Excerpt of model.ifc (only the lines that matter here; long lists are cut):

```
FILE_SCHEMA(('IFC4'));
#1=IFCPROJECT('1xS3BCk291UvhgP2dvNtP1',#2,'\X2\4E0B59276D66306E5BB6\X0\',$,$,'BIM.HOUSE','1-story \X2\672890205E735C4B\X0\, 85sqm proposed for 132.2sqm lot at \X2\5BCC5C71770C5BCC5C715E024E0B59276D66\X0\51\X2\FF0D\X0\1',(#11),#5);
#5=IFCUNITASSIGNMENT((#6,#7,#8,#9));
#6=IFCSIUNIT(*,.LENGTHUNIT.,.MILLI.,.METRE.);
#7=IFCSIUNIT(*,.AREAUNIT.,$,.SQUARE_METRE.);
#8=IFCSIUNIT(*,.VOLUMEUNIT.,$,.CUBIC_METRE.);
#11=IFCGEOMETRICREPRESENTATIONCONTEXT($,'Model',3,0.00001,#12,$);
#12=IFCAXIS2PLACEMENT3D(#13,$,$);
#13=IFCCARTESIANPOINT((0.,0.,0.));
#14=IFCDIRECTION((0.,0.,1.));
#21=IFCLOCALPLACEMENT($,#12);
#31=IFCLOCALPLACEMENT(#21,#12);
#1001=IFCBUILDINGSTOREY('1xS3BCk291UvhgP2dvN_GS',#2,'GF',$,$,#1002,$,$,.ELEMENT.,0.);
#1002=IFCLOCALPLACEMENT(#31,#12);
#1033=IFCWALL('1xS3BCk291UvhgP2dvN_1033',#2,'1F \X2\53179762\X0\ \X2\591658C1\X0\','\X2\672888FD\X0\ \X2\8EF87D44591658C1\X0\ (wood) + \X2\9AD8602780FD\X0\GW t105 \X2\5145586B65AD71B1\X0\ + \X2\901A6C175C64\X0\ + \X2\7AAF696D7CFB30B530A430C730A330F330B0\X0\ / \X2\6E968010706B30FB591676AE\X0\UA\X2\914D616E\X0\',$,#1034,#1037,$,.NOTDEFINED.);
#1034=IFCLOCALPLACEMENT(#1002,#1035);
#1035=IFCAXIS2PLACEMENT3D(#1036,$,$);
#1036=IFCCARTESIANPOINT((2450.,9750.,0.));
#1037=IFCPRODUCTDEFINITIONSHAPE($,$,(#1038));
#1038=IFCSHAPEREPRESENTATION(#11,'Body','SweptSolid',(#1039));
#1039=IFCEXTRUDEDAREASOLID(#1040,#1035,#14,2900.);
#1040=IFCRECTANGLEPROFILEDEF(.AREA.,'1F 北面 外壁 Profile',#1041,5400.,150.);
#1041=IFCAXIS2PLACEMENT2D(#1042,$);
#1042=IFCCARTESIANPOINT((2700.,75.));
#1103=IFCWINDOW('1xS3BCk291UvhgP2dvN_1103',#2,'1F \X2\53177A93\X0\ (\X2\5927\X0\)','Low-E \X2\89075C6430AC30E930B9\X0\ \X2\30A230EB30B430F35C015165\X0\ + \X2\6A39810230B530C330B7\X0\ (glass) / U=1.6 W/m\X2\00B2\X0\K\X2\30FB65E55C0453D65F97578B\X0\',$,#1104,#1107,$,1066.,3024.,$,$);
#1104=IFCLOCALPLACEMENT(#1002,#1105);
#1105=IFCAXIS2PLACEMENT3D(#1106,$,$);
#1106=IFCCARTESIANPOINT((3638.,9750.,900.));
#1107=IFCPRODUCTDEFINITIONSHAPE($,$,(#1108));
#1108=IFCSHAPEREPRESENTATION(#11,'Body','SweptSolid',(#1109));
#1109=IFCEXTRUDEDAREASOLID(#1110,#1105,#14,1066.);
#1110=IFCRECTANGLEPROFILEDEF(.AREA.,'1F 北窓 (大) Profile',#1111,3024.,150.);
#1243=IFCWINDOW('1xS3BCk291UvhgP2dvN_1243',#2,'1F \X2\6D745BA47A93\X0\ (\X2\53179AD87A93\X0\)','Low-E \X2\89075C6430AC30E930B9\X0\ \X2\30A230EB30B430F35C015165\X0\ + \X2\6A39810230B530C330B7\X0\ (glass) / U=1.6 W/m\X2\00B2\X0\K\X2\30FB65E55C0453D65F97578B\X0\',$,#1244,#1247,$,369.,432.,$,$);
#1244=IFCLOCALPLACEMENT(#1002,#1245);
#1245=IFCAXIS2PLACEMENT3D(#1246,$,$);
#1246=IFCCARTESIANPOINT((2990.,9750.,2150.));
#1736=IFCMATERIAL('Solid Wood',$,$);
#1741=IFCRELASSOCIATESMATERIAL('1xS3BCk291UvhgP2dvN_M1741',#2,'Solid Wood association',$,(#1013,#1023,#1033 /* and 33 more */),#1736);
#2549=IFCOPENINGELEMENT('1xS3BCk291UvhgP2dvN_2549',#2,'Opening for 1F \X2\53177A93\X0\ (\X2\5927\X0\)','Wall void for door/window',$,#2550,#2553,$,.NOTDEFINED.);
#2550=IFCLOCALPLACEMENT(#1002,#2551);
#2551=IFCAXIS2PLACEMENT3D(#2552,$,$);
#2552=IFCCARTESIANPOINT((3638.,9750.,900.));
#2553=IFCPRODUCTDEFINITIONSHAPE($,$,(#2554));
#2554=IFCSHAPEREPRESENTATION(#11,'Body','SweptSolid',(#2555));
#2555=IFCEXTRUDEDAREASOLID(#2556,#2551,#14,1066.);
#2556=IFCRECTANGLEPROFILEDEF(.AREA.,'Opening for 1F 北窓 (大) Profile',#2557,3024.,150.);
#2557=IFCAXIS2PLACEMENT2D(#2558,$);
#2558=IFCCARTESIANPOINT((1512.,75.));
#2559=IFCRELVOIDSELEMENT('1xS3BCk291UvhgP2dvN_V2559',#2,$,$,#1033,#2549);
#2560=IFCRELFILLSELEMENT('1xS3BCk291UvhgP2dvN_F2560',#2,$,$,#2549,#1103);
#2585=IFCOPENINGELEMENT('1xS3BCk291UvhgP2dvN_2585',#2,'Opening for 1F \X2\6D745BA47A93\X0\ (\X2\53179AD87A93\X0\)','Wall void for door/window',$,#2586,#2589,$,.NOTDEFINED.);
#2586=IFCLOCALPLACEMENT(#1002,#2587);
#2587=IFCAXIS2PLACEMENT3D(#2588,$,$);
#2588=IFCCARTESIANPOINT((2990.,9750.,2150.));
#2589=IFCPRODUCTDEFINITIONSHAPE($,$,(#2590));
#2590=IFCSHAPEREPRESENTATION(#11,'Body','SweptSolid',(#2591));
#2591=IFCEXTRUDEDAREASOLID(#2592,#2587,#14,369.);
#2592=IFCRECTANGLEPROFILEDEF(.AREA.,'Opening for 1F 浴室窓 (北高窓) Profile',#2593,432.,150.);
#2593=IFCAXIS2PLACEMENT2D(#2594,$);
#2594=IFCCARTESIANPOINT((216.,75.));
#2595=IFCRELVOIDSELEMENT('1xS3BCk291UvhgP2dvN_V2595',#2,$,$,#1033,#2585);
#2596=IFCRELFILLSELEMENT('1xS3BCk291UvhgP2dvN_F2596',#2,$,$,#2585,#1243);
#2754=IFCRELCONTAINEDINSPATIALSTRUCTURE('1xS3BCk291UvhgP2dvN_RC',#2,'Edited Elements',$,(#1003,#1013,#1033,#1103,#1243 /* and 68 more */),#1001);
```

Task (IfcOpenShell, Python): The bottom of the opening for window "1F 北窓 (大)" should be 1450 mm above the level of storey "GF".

```python
import numpy as np
import ifcopenshell
import ifcopenshell.api.geometry
import ifcopenshell.geom
import ifcopenshell.util.element
import ifcopenshell.util.placement
import ifcopenshell.util.shape
import ifcopenshell.util.unit

model = ifcopenshell.open("model.ifc")
unit_scale = ifcopenshell.util.unit.calculate_unit_scale(model)

window = model.by_guid("1xS3BCk291UvhgP2dvN_1103")
opening = window.FillsVoids[0].RelatingOpeningElement
storey = ifcopenshell.util.element.get_container(window, ifc_class="IfcBuildingStorey")
level = ifcopenshell.util.placement.get_local_placement(storey.ObjectPlacement)[2, 3]

# The opening's origin need not be at the sill, so measure its lowest point.
shape = ifcopenshell.geom.create_shape(ifcopenshell.geom.settings(), opening)
bottom = ifcopenshell.util.shape.get_shape_bottom_elevation(shape, shape.geometry) / unit_scale
dz = level + 1450.0 - bottom

shift = np.array([0.0, 0.0, dz])
# The window is not placed relative to its opening, so move both.
for product in (opening, window):
    matrix = ifcopenshell.util.placement.get_local_placement(product.ObjectPlacement)
    matrix[:3, 3] += shift
    ifcopenshell.api.geometry.edit_object_placement(model, product=product, matrix=matrix, is_si=False)

print(f"moved by {dz * unit_scale:+.3f} m")

model.write("model_updated.ifc")
```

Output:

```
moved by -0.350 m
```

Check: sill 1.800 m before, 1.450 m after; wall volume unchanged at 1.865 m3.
